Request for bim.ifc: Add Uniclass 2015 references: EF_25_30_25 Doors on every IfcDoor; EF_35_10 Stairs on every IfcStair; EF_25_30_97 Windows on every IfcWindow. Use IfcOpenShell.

First a look at what the model holds.

```python
import ifcopenshell

model = ifcopenshell.open("bim.ifc")
print(model.schema)
print("classifications:", [c.Name for c in model.by_type("IfcClassification")])
for ifc_class in ("IfcDoor", "IfcRoof", "IfcStair", "IfcWall", "IfcWindow"):
    print(ifc_class, len(model.by_type(ifc_class)))
```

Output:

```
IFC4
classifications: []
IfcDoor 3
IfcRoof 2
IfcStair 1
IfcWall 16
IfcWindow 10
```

```python
import ifcopenshell
import ifcopenshell.api.classification

model = ifcopenshell.open("bim.ifc")

system = ifcopenshell.api.classification.add_classification(model, classification="Uniclass 2015")

codes = {
    "IfcDoor": ("EF_25_30_25", "Doors"),
    "IfcStair": ("EF_35_10", "Stairs"),
    "IfcWindow": ("EF_25_30_97", "Windows"),
}
for ifc_class, (code, name) in codes.items():
    products = model.by_type(ifc_class)
    ifcopenshell.api.classification.add_reference(
        model, products=products, classification=system, identification=code, name=name
    )
    print(code, len(products))

model.write("bim_rev.ifc")
```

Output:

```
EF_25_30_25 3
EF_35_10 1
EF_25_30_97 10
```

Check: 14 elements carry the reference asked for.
